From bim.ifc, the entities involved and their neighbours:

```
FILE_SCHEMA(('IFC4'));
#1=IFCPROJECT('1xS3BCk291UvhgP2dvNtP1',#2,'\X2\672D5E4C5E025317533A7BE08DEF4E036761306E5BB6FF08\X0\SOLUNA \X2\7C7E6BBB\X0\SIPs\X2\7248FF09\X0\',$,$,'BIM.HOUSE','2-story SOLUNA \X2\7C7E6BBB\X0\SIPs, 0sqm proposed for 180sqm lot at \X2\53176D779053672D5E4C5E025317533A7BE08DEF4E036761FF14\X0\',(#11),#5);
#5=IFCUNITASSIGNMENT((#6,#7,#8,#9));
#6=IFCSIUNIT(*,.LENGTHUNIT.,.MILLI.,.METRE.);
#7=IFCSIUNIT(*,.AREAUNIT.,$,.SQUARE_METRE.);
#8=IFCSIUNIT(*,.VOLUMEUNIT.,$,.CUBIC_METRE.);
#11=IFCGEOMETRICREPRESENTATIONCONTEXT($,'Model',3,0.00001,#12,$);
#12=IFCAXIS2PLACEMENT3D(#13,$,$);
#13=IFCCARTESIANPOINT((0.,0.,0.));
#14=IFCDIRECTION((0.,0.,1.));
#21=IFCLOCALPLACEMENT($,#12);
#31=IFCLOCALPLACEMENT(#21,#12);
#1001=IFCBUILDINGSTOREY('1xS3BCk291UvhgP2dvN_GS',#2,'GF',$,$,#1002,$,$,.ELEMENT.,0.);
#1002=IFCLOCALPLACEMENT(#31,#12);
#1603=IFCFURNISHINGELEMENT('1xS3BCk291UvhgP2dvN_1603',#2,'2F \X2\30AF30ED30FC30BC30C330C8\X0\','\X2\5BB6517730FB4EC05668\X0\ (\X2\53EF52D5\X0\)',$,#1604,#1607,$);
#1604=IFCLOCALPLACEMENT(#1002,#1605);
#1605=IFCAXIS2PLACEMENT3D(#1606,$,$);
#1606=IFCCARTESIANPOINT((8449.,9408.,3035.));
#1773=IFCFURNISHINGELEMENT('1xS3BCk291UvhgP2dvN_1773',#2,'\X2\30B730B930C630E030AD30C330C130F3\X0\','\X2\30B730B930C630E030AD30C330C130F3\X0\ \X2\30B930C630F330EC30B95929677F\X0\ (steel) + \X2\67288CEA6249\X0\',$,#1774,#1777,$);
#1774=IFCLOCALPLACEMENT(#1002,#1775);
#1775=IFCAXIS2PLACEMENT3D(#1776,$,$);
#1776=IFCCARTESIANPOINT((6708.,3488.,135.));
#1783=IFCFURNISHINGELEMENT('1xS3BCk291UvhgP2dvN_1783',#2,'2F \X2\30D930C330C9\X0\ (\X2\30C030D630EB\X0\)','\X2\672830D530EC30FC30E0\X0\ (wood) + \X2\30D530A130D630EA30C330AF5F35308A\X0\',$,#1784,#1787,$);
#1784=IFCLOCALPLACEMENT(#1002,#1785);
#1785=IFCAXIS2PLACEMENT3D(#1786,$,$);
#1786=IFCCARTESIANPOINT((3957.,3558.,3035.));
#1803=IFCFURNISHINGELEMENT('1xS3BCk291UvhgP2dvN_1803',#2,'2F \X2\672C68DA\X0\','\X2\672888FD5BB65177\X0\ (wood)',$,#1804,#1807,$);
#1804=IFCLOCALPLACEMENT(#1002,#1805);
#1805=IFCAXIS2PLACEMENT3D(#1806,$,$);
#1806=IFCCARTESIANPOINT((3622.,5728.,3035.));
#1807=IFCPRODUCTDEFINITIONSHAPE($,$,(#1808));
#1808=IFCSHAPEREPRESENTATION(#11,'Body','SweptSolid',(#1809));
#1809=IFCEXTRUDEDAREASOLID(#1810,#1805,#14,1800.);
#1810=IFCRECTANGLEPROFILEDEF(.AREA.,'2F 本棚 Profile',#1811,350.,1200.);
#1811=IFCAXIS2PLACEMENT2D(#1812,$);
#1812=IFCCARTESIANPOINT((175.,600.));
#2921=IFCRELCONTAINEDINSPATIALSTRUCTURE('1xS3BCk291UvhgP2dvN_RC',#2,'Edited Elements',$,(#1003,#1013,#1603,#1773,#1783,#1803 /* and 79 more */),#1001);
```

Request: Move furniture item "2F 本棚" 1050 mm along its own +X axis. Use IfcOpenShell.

```python
import ifcopenshell
import ifcopenshell.api.geometry
import ifcopenshell.util.placement
import ifcopenshell.util.unit

model = ifcopenshell.open("bim.ifc")
unit_scale = ifcopenshell.util.unit.calculate_unit_scale(model)

item = model.by_guid("1xS3BCk291UvhgP2dvN_1803")
matrix = ifcopenshell.util.placement.get_local_placement(item.ObjectPlacement)
matrix[:3, 3] += matrix[:3, 0] * 1.05 / unit_scale
ifcopenshell.api.geometry.edit_object_placement(model, product=item, matrix=matrix, is_si=False)

print(ifcopenshell.util.placement.get_local_placement(item.ObjectPlacement).round(3) + 0.0)

model.write("bim_v2.ifc")
```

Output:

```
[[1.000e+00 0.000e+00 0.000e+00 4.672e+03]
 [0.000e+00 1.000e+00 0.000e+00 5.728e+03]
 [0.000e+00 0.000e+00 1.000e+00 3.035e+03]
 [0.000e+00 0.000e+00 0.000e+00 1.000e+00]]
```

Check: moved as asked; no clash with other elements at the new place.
